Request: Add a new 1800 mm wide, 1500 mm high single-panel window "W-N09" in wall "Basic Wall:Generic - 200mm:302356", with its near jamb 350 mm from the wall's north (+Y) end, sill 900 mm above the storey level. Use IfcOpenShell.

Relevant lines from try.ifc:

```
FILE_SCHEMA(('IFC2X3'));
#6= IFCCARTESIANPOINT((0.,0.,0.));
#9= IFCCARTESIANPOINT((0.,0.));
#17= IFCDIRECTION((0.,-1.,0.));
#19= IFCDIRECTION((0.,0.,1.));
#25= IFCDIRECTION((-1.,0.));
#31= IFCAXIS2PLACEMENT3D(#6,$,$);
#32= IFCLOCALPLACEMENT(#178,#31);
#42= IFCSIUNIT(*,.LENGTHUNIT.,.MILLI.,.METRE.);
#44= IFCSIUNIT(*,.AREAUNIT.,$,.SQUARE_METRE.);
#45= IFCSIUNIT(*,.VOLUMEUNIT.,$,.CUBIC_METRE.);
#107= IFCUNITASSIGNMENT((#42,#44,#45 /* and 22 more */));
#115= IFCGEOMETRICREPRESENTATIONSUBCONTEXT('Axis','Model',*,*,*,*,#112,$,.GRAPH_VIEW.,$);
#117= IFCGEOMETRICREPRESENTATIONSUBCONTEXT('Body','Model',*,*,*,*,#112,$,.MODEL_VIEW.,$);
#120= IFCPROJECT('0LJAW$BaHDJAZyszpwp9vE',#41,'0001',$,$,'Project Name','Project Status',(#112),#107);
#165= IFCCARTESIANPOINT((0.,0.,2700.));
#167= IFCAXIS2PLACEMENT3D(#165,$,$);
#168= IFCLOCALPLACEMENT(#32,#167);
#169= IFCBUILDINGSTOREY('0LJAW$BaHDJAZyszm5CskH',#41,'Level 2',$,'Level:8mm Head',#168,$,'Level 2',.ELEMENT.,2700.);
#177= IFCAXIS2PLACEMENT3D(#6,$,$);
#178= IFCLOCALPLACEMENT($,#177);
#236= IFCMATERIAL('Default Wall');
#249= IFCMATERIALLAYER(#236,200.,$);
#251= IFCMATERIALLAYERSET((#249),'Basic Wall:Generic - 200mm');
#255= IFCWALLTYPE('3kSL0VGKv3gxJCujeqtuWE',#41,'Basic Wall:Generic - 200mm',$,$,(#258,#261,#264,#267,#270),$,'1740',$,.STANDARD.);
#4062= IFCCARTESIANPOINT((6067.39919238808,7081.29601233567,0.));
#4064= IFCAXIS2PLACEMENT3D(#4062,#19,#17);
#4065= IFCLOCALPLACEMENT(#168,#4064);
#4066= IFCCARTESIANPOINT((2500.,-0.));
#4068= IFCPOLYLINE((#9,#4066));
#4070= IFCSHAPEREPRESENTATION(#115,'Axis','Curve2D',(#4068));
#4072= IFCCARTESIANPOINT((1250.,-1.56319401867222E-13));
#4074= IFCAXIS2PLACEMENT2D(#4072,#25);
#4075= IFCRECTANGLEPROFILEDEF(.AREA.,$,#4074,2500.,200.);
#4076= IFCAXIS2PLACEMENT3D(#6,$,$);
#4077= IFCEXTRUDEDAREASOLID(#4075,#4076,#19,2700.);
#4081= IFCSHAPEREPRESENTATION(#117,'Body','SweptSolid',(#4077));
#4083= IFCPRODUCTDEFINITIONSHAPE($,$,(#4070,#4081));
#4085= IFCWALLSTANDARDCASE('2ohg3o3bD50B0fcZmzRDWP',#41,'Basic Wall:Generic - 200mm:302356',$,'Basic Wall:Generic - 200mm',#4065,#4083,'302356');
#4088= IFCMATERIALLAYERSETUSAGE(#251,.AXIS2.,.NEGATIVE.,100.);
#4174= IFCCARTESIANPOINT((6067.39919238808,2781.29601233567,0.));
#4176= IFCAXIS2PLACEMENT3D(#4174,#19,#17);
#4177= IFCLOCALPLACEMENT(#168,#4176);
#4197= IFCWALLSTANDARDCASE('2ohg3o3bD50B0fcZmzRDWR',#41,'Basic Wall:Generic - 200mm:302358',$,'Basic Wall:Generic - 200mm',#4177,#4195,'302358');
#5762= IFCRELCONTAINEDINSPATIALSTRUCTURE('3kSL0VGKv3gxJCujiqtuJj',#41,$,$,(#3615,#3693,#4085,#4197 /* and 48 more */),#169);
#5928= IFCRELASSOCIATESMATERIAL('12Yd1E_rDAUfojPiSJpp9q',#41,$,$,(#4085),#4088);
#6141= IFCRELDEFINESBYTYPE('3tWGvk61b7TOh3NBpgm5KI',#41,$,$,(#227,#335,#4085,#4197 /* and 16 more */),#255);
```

```python
import numpy as np
import ifcopenshell
import ifcopenshell.api.feature
import ifcopenshell.api.geometry
import ifcopenshell.api.root
import ifcopenshell.api.spatial
import ifcopenshell.api.type
import ifcopenshell.geom
import ifcopenshell.util.element
import ifcopenshell.util.placement
import ifcopenshell.util.representation
import ifcopenshell.util.shape
import ifcopenshell.util.unit

model = ifcopenshell.open("try.ifc")
unit_scale = ifcopenshell.util.unit.calculate_unit_scale(model)
settings = ifcopenshell.geom.settings()


def volume(element):
    """Net volume in cubic metres, openings subtracted."""
    shape = ifcopenshell.geom.create_shape(settings, element)
    return ifcopenshell.util.shape.get_volume(shape.geometry)


wall = model.by_id(4085)
storey = ifcopenshell.util.element.get_container(wall, ifc_class="IfcBuildingStorey")
context = ifcopenshell.util.representation.get_context(model, "Model", "Body", "MODEL_VIEW")
before = volume(wall)

width, height, from_end, sill = 1.8, 1.5, 0.35, 0.9  # metres

# The wall runs along its own X axis, and the end named is its -X end.
wall_shape = ifcopenshell.geom.create_shape(settings, wall)
x, y, z = ifcopenshell.util.shape.get_vertices(wall_shape.geometry).T
start = x.min() + from_end
face, thickness = float(y.min()), float(y.max() - y.min())
wall_matrix = ifcopenshell.util.placement.get_local_placement(wall.ObjectPlacement)
level = ifcopenshell.util.placement.get_local_placement(storey.ObjectPlacement)[2, 3]


def in_wall(x, y):
    """Placement at x, y metres in the wall's axes, at sill height."""
    matrix = wall_matrix.copy()
    matrix[:, 3] = wall_matrix @ np.array([x / unit_scale, y / unit_scale, 0.0, 1.0])
    matrix[2, 3] = level + sill / unit_scale
    return matrix


# Opening: a box that overshoots both wall faces by 50 mm.
opening = ifcopenshell.api.root.create_entity(model, ifc_class="IfcOpeningElement")
box = ifcopenshell.api.geometry.add_wall_representation(
    model, context=context, length=width, height=height, thickness=thickness + 0.1
)
ifcopenshell.api.geometry.assign_representation(model, product=opening, representation=box)
ifcopenshell.api.geometry.edit_object_placement(model, product=opening, matrix=in_wall(start, face - 0.05), is_si=False)
ifcopenshell.api.feature.add_feature(model, feature=opening, element=wall)

window = ifcopenshell.api.root.create_entity(model, ifc_class="IfcWindow", name="W-N09")
window.OverallWidth, window.OverallHeight = width / unit_scale, height / unit_scale
body = ifcopenshell.api.geometry.add_window_representation(
    model,
    context=context,
    overall_width=window.OverallWidth,
    overall_height=window.OverallHeight,
    partition_type="SINGLE_PANEL",
)
ifcopenshell.api.geometry.assign_representation(model, product=window, representation=body)
ifcopenshell.api.spatial.assign_container(model, products=[window], relating_structure=storey)
fills = ifcopenshell.api.feature.add_filling(model, opening=opening, element=window)
fills.OwnerHistory = window.OwnerHistory  # required in IFC2X3

# IFC2X3 keeps the operation on the window style.
style = ifcopenshell.api.root.create_entity(model, ifc_class="IfcWindowStyle", name="W-N09")
style.OperationType, style.ConstructionType = "SINGLE_PANEL", "NOTDEFINED"
style.ParameterTakesPrecedence = style.Sizeable = False
ifcopenshell.api.type.assign_type(model, related_objects=[window], relating_type=style)

# Centre the window in the wall's thickness.
ifcopenshell.api.geometry.edit_object_placement(model, product=window, matrix=in_wall(start, face), is_si=False)
window_shape = ifcopenshell.geom.create_shape(settings, window)
depth = ifcopenshell.util.shape.get_vertices(window_shape.geometry)[:, 1]
offset = face + thickness / 2 - (depth.min() + depth.max()) / 2
ifcopenshell.api.geometry.edit_object_placement(model, product=window, matrix=in_wall(start, offset), is_si=False)

after = volume(wall)

print(f"wall volume {before:.3f} -> {after:.3f} m3")

model.write("try_v2.ifc")
```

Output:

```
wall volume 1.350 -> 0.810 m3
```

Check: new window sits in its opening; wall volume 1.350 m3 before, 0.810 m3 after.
